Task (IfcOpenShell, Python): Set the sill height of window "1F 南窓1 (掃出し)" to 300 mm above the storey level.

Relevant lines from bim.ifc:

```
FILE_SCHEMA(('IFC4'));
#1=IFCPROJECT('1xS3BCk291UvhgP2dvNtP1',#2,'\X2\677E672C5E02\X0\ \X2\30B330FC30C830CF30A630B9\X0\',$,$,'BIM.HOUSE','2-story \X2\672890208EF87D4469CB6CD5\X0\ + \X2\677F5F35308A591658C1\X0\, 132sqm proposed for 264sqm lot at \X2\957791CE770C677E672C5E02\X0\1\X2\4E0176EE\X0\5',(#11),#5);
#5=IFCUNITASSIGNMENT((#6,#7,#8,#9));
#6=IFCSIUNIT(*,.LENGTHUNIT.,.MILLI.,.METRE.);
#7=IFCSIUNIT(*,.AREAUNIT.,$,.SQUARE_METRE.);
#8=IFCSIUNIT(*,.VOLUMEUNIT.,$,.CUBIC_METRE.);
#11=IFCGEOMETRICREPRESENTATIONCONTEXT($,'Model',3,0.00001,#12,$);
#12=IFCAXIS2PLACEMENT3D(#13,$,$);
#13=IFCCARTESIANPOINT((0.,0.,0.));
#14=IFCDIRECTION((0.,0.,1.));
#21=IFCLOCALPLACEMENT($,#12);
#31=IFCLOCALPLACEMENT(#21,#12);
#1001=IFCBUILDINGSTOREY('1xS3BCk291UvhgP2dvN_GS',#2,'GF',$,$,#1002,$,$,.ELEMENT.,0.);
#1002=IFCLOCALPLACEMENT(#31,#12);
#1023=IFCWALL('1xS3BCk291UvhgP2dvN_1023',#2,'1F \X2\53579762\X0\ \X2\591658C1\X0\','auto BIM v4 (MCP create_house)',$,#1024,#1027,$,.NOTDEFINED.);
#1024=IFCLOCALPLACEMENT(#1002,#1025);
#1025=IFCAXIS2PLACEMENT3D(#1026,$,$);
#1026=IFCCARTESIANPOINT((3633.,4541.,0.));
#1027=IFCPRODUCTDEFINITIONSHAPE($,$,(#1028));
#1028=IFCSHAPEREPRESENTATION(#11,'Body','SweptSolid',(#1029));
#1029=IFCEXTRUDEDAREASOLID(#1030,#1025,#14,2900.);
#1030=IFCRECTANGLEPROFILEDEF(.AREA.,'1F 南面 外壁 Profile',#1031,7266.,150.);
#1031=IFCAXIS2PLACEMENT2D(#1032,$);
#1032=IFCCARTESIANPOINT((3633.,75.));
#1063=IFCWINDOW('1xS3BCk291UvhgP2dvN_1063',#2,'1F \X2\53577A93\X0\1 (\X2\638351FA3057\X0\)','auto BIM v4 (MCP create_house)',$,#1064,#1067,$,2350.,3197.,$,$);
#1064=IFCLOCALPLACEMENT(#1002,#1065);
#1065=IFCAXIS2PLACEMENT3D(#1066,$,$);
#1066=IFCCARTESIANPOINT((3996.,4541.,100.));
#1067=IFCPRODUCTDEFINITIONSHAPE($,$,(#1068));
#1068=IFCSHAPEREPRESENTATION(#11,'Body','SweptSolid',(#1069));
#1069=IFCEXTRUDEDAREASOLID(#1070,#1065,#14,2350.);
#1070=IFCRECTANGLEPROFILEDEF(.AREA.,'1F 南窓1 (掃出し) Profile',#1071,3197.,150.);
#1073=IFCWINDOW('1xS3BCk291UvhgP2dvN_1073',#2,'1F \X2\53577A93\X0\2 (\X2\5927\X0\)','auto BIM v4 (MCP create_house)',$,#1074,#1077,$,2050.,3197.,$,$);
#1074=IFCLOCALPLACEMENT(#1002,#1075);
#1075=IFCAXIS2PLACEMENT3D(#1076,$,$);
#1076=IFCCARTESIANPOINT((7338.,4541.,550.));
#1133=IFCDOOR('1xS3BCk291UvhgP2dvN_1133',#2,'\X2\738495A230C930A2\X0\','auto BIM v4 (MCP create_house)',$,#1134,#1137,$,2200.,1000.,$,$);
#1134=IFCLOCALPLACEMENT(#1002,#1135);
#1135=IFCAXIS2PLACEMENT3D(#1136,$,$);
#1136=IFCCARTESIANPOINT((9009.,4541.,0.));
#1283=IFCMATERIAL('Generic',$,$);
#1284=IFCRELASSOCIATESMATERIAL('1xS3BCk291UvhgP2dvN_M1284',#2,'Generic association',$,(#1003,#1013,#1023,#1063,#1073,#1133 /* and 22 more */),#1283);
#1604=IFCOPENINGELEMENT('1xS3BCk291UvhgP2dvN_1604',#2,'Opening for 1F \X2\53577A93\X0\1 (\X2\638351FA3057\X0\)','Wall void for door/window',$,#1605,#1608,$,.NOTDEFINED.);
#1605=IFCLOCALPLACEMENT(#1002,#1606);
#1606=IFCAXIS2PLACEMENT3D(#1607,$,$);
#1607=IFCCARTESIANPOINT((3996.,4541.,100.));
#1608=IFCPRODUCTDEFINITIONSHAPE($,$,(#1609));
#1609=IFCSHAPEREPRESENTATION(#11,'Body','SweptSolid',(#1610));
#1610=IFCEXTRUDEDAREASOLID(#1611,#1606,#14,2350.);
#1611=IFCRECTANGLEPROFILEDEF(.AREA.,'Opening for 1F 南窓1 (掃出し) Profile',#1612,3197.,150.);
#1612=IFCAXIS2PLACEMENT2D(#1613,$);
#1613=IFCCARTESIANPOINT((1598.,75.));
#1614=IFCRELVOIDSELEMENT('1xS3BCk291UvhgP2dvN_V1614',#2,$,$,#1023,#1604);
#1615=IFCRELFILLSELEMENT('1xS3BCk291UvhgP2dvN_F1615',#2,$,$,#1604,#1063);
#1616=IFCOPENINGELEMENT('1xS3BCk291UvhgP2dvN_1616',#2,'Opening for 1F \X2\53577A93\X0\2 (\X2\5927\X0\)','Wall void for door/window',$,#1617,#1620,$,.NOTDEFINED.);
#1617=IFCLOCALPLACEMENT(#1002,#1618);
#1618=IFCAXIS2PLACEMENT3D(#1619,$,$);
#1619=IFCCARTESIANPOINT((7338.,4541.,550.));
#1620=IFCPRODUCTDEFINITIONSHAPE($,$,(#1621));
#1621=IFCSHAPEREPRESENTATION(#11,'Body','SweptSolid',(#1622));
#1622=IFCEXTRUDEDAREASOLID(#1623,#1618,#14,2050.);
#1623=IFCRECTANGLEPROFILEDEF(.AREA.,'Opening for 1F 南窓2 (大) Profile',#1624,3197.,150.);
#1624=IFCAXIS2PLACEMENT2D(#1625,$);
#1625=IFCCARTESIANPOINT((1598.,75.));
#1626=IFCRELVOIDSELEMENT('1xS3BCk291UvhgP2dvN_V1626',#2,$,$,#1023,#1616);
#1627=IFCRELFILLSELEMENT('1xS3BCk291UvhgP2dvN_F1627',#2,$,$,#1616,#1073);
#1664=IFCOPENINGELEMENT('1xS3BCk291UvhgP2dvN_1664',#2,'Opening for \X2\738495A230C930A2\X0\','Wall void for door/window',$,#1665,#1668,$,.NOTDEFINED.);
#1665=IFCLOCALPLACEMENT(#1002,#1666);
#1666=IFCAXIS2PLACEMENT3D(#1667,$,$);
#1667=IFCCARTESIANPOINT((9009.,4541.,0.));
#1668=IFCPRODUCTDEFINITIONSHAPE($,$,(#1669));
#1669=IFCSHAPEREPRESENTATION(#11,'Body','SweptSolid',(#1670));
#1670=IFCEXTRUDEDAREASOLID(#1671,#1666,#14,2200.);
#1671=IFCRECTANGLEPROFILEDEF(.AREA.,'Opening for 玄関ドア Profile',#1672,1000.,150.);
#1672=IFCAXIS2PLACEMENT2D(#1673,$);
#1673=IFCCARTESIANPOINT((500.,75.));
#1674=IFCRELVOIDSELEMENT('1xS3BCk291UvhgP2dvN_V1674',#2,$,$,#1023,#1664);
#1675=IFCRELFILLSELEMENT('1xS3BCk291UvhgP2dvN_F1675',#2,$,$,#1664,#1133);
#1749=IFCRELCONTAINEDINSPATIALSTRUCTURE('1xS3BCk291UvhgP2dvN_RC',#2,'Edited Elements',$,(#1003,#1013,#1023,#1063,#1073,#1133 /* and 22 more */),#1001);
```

```python
import numpy as np
import ifcopenshell
import ifcopenshell.api.geometry
import ifcopenshell.geom
import ifcopenshell.util.element
import ifcopenshell.util.placement
import ifcopenshell.util.shape
import ifcopenshell.util.unit

model = ifcopenshell.open("bim.ifc")
unit_scale = ifcopenshell.util.unit.calculate_unit_scale(model)

window = model.by_id(1063)
opening = window.FillsVoids[0].RelatingOpeningElement
storey = ifcopenshell.util.element.get_container(window, ifc_class="IfcBuildingStorey")
level = ifcopenshell.util.placement.get_local_placement(storey.ObjectPlacement)[2, 3]

# The opening's origin need not be at the sill, so measure its lowest point.
shape = ifcopenshell.geom.create_shape(ifcopenshell.geom.settings(), opening)
bottom = ifcopenshell.util.shape.get_shape_bottom_elevation(shape, shape.geometry) / unit_scale
dz = level + 0.3 / unit_scale - bottom

shift = np.array([0.0, 0.0, dz])
# The window is not placed relative to its opening, so move both.
for product in (opening, window):
    matrix = ifcopenshell.util.placement.get_local_placement(product.ObjectPlacement)
    matrix[:3, 3] += shift
    ifcopenshell.api.geometry.edit_object_placement(model, product=product, matrix=matrix, is_si=False)

print(f"moved by {dz * unit_scale:+.3f} m")

model.write("bim-out.ifc")
```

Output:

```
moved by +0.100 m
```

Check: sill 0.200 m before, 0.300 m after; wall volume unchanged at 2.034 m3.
